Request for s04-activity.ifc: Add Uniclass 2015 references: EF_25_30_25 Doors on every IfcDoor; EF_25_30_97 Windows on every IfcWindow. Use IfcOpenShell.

First a look at what the model holds.

```python
import ifcopenshell

model = ifcopenshell.open("s04-activity.ifc")
print(model.schema)
print("classifications:", [c.Name for c in model.by_type("IfcClassification")])
for ifc_class in ("IfcDoor", "IfcRoof", "IfcStair", "IfcWall", "IfcWindow"):
    print(ifc_class, len(model.by_type(ifc_class)))
```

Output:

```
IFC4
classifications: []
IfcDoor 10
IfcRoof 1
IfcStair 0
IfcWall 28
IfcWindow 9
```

```python
import ifcopenshell
import ifcopenshell.api.classification

model = ifcopenshell.open("s04-activity.ifc")

system = ifcopenshell.api.classification.add_classification(model, classification="Uniclass 2015")

codes = {
    "IfcDoor": ("EF_25_30_25", "Doors"),
    "IfcWindow": ("EF_25_30_97", "Windows"),
}
for ifc_class, (code, name) in codes.items():
    products = model.by_type(ifc_class)
    ifcopenshell.api.classification.add_reference(
        model, products=products, classification=system, identification=code, name=name
    )
    print(code, len(products))

model.write("s04-activity-out.ifc")
```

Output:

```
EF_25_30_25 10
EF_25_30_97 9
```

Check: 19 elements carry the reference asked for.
